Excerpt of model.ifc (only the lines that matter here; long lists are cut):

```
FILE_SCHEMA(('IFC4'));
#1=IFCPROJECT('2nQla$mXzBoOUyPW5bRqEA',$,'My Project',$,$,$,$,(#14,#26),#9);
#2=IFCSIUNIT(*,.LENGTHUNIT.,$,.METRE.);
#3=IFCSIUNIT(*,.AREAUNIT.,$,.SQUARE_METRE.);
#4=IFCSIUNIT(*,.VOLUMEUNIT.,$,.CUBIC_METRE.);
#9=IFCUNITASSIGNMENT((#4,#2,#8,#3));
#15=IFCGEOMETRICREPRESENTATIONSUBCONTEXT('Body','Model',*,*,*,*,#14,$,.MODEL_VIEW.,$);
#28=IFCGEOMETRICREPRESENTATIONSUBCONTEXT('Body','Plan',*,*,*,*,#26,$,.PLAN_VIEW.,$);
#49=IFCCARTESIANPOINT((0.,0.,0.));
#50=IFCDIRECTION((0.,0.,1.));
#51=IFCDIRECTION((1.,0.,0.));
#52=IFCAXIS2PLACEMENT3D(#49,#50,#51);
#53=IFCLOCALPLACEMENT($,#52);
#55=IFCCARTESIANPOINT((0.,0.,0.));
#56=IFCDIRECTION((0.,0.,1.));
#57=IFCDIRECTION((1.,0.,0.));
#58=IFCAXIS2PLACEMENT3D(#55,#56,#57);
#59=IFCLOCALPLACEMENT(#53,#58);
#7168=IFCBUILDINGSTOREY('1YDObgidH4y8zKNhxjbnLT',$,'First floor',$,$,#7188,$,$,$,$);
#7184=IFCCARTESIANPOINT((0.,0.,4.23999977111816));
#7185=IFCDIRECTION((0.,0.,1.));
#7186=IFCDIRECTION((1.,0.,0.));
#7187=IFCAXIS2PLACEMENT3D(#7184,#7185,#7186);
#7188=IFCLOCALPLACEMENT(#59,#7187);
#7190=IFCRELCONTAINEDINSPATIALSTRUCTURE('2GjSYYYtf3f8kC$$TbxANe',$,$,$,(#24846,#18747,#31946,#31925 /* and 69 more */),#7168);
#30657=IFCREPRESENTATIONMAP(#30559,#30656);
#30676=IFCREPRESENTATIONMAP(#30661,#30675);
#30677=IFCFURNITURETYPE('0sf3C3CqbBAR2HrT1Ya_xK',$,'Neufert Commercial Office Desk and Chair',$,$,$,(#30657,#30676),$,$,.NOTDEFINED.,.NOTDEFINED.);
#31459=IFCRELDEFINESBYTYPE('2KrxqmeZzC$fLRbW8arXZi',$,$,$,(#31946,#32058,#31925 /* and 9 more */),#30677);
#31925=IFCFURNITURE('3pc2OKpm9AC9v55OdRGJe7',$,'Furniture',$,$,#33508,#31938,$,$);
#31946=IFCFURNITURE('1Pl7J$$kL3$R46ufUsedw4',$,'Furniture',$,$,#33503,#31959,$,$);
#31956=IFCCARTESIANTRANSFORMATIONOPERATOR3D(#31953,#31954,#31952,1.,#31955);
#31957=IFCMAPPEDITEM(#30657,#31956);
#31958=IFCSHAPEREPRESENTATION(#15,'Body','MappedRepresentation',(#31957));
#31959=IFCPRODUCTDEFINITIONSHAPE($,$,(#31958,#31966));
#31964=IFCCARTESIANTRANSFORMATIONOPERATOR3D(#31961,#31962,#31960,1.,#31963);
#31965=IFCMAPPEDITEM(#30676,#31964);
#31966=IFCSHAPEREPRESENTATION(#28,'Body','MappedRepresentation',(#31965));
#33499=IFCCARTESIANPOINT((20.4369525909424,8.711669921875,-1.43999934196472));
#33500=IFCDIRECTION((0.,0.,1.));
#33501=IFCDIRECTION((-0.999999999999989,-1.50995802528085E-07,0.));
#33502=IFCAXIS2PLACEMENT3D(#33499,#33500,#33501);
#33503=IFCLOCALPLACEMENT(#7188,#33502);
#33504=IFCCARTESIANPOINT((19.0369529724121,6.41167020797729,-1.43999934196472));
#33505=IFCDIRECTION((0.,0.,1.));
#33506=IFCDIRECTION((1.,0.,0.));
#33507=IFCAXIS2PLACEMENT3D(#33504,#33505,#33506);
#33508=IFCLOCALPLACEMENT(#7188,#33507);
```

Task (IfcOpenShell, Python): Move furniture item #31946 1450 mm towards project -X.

```python
import ifcopenshell
import ifcopenshell.api.geometry
import ifcopenshell.util.placement
import ifcopenshell.util.unit

model = ifcopenshell.open("model.ifc")
unit_scale = ifcopenshell.util.unit.calculate_unit_scale(model)

item = model.by_guid("1Pl7J$$kL3$R46ufUsedw4")
matrix = ifcopenshell.util.placement.get_local_placement(item.ObjectPlacement)
matrix[0, 3] -= 1.45 / unit_scale
ifcopenshell.api.geometry.edit_object_placement(model, product=item, matrix=matrix, is_si=False)

print(ifcopenshell.util.placement.get_local_placement(item.ObjectPlacement).round(3) + 0.0)

model.write("model_v2.ifc")
```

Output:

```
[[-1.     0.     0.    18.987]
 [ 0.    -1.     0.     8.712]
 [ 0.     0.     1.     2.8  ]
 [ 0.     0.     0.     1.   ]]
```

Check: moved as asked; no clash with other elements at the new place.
